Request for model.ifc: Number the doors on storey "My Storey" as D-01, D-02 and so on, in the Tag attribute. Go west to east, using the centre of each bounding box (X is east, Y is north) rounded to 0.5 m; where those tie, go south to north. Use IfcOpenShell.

First a look at what the model holds.

```python
import ifcopenshell
import ifcopenshell.util.element
import ifcopenshell.util.placement

model = ifcopenshell.open("model.ifc")
print(model.schema)
storey = next(s for s in model.by_type("IfcBuildingStorey") if s.Name == "My Storey")
doors = [e for e in ifcopenshell.util.element.get_decomposition(storey) if e.is_a("IfcDoor")]
for e in sorted(doors, key=lambda e: e.id()):
    origin = ifcopenshell.util.placement.get_local_placement(e.ObjectPlacement)[:3, 3]
    print(e.id(), e.Tag, e.Name, origin.round(2) + 0.0, sep=" | ")
```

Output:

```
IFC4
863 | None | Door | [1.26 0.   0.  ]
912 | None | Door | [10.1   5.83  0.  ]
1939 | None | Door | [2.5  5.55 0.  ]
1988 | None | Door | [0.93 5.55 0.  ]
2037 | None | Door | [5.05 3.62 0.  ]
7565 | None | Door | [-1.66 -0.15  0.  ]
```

```python
import ifcopenshell
import ifcopenshell.geom
import ifcopenshell.util.element
import ifcopenshell.util.shape

model = ifcopenshell.open("model.ifc")
settings = ifcopenshell.geom.settings()
settings.set("use-world-coords", True)


def centre(element):
    shape = ifcopenshell.geom.create_shape(settings, element)
    return ifcopenshell.util.shape.get_bbox_centroid(shape.geometry)


storey = next(s for s in model.by_type("IfcBuildingStorey") if s.Name == "My Storey")
doors = [e for e in ifcopenshell.util.element.get_decomposition(storey) if e.is_a("IfcDoor")]

# Insertion points can sit at a corner or the storey origin, so sort by the geometry (in metres).
centres = {e: centre(e) for e in doors}
doors.sort(key=lambda e: (round(centres[e][0] / 0.5), centres[e][1]))

for i, e in enumerate(doors, start=1):
    number = f"D-{i:02d}"
    e.Tag = number
    print(e.id(), number)

model.write("model_v2.ifc")
```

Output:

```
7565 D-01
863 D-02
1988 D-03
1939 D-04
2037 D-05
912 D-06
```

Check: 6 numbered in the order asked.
